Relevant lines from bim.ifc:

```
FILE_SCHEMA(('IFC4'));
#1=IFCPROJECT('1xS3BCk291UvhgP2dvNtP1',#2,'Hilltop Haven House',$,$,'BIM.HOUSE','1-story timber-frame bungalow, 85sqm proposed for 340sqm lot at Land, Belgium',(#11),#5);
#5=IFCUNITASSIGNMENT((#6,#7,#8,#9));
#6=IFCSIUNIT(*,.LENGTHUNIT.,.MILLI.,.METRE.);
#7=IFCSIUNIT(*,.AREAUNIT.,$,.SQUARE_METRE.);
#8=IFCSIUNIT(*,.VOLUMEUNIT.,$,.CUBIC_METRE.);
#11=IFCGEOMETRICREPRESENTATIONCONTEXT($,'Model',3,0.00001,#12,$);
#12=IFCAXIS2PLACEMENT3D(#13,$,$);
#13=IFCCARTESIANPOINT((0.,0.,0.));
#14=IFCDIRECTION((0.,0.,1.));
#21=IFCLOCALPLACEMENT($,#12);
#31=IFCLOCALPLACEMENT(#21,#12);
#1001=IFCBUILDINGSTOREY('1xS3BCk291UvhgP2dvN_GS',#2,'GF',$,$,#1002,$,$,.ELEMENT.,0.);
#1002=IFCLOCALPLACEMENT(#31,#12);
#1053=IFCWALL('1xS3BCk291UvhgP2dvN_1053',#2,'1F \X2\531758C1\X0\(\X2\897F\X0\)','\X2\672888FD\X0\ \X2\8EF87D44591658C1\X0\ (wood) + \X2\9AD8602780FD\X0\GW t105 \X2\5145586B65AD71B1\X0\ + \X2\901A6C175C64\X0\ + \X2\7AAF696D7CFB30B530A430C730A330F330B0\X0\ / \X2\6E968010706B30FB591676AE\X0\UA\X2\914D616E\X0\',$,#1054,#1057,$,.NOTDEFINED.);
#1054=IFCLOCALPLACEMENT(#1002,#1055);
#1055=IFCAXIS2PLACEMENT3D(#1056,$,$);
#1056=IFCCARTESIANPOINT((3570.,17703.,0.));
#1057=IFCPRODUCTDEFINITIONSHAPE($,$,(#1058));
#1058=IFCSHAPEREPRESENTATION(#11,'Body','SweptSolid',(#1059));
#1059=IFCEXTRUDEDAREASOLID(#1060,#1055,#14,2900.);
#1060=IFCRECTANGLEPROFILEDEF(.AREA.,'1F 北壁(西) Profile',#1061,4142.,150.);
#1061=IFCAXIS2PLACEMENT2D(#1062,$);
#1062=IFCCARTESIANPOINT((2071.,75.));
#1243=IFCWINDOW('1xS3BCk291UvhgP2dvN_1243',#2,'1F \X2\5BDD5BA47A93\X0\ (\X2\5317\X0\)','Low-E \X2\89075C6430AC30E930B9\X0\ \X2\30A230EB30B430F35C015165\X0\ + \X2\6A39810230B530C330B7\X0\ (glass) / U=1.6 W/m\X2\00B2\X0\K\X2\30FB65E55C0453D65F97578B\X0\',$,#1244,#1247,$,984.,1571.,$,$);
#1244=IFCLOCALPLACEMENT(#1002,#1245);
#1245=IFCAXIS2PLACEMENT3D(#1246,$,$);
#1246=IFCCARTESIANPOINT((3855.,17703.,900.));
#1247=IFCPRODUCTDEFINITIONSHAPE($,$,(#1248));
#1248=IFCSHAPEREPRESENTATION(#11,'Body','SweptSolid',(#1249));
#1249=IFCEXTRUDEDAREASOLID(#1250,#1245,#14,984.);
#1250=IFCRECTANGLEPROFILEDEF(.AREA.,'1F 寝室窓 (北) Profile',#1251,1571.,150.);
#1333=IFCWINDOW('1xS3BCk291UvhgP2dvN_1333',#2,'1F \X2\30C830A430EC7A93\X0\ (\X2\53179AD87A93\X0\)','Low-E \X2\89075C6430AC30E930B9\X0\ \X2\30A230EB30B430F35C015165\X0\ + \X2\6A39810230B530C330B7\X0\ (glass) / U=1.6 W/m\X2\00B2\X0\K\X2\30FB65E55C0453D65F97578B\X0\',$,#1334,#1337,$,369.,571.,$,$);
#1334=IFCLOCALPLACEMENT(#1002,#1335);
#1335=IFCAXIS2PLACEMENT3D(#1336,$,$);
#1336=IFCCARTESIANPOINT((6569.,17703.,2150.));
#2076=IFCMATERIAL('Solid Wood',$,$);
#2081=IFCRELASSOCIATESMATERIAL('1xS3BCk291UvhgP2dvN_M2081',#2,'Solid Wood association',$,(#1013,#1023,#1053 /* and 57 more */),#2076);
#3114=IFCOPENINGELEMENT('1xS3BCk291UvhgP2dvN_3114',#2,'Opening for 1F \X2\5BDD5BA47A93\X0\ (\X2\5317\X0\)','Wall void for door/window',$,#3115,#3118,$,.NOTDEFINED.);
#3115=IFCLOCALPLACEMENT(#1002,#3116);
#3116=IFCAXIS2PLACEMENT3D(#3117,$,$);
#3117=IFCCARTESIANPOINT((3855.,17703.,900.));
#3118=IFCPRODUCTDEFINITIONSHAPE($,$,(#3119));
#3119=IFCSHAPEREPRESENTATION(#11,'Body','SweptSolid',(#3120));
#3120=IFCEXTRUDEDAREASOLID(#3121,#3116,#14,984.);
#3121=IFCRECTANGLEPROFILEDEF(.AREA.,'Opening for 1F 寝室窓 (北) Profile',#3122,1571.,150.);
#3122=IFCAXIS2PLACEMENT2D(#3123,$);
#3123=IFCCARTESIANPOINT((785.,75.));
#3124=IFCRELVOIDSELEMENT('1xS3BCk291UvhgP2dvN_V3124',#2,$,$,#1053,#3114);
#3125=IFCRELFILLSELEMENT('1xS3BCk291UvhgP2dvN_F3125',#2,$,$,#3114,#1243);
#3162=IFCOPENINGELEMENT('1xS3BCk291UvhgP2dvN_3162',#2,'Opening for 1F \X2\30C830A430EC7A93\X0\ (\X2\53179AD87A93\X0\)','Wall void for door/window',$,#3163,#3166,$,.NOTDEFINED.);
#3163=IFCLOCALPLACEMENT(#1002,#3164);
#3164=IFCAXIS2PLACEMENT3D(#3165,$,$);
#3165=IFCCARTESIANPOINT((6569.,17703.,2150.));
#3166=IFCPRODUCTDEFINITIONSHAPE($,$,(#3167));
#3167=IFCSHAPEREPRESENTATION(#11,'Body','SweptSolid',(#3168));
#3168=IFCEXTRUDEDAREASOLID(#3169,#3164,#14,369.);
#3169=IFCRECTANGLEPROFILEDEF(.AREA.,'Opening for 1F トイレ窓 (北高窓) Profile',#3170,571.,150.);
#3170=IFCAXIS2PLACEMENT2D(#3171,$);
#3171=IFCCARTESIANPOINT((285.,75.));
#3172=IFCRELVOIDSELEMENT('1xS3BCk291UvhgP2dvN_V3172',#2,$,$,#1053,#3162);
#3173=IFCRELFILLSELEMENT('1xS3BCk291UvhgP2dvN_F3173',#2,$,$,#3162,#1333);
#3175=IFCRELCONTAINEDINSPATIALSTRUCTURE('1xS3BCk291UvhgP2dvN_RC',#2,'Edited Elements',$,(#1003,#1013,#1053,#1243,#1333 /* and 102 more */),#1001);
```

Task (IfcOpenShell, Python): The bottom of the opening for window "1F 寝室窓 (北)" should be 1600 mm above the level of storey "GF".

```python
import numpy as np
import ifcopenshell
import ifcopenshell.api.geometry
import ifcopenshell.geom
import ifcopenshell.util.element
import ifcopenshell.util.placement
import ifcopenshell.util.shape
import ifcopenshell.util.unit

model = ifcopenshell.open("bim.ifc")
unit_scale = ifcopenshell.util.unit.calculate_unit_scale(model)

window = model.by_guid("1xS3BCk291UvhgP2dvN_1243")
opening = window.FillsVoids[0].RelatingOpeningElement
storey = ifcopenshell.util.element.get_container(window, ifc_class="IfcBuildingStorey")
level = ifcopenshell.util.placement.get_local_placement(storey.ObjectPlacement)[2, 3]

# The opening's origin need not be at the sill, so measure its lowest point.
shape = ifcopenshell.geom.create_shape(ifcopenshell.geom.settings(), opening)
bottom = ifcopenshell.util.shape.get_shape_bottom_elevation(shape, shape.geometry) / unit_scale
dz = level + 1.6 / unit_scale - bottom

shift = np.array([0.0, 0.0, dz])
# The window is not placed relative to its opening, so move both.
for product in (opening, window):
    matrix = ifcopenshell.util.placement.get_local_placement(product.ObjectPlacement)
    matrix[:3, 3] += shift
    ifcopenshell.api.geometry.edit_object_placement(model, product=product, matrix=matrix, is_si=False)

print(f"moved by {dz * unit_scale:+.3f} m")

model.write("bim-out.ifc")
```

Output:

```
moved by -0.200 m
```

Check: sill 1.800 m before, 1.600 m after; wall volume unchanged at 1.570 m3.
